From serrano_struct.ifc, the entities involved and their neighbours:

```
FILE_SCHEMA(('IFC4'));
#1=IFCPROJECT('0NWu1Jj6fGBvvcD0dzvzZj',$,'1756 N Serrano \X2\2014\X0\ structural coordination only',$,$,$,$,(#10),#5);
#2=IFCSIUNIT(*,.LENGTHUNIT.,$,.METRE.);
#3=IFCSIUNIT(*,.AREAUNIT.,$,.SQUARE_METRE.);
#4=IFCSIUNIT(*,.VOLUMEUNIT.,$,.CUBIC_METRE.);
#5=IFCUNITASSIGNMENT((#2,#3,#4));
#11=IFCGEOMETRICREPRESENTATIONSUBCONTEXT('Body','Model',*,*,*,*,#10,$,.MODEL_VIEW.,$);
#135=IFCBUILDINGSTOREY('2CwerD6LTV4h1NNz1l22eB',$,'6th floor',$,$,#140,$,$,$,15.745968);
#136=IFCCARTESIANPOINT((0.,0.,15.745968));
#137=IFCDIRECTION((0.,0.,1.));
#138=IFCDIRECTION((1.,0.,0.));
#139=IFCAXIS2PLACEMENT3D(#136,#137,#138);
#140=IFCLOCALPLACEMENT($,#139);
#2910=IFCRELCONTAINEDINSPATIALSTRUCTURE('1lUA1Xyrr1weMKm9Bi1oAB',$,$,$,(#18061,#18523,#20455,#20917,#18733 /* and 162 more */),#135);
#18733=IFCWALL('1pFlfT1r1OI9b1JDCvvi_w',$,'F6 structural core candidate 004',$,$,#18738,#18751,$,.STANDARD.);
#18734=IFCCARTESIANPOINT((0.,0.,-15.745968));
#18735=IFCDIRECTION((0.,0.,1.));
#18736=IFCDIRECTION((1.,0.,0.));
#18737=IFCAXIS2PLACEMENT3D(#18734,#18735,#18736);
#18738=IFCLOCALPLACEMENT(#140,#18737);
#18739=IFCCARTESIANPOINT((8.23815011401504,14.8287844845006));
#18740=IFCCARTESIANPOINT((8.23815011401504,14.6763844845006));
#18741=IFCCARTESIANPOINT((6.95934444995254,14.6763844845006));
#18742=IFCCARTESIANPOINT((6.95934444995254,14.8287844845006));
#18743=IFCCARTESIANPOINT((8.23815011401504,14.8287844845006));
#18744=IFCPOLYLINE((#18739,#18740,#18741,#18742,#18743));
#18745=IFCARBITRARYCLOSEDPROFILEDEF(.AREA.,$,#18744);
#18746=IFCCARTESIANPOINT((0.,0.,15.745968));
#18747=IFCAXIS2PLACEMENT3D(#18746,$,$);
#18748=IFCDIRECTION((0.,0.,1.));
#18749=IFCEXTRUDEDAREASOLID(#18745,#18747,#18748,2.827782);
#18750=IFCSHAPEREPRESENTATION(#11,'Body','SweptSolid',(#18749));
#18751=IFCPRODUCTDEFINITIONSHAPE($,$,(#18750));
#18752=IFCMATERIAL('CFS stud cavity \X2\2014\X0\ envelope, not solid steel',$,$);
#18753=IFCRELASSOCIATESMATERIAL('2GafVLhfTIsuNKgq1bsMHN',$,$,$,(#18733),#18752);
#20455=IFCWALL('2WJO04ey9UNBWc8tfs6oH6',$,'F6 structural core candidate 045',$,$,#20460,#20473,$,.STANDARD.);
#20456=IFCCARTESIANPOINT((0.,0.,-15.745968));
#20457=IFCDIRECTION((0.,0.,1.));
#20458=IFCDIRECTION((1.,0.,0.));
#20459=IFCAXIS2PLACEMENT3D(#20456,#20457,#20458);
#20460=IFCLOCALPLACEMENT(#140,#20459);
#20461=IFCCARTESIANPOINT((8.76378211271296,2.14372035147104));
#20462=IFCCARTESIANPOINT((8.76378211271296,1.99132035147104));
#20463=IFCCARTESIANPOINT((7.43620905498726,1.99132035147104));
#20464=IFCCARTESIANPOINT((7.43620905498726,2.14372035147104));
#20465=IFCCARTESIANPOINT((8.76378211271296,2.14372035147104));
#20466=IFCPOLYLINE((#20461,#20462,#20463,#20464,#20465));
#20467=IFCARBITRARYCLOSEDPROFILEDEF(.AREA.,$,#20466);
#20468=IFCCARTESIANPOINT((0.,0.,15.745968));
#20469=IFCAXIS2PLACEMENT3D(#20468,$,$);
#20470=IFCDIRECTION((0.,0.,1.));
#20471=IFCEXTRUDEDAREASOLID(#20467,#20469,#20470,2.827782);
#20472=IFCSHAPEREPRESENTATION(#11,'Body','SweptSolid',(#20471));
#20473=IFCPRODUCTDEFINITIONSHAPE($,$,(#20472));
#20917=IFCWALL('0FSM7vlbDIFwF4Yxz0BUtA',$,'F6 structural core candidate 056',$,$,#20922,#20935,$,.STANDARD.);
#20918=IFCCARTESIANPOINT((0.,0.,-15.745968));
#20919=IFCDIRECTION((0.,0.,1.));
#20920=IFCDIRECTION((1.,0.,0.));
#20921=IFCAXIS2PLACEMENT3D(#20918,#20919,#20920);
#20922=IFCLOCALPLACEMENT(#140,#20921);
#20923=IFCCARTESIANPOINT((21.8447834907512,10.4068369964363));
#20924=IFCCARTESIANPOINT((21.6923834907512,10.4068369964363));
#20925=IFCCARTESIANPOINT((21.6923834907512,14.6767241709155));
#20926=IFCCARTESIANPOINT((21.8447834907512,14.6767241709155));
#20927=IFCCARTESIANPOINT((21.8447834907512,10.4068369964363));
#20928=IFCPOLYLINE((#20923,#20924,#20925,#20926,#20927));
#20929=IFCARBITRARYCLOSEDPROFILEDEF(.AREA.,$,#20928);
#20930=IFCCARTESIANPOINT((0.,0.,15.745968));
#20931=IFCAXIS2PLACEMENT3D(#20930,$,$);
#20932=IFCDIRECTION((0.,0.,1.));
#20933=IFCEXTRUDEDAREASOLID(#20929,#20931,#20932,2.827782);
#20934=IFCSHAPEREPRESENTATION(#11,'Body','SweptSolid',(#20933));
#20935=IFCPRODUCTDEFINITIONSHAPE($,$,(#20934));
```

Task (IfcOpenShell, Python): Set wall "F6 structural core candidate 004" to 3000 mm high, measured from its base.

```python
import ifcopenshell
import ifcopenshell.geom
import ifcopenshell.util.representation
import ifcopenshell.util.shape

model = ifcopenshell.open("serrano_struct.ifc")
settings = ifcopenshell.geom.settings()


def volume(element):
    """Net volume in cubic metres, openings subtracted."""
    shape = ifcopenshell.geom.create_shape(settings, element)
    return ifcopenshell.util.shape.get_volume(shape.geometry)


wall = model.by_guid("1pFlfT1r1OI9b1JDCvvi_w")
before = volume(wall)

body = ifcopenshell.util.representation.get_representation(wall, "Model", "Body")
solid = body.Items[0]
old_height = solid.Depth
solid.Depth = 3.0
after = volume(wall)

print(f"height {old_height:g} -> {solid.Depth:g}, volume {before:.3f} -> {after:.3f} m3")

model.write("serrano_struct_edited.ifc")
```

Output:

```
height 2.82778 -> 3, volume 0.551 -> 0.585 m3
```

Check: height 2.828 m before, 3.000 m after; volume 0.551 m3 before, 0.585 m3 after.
